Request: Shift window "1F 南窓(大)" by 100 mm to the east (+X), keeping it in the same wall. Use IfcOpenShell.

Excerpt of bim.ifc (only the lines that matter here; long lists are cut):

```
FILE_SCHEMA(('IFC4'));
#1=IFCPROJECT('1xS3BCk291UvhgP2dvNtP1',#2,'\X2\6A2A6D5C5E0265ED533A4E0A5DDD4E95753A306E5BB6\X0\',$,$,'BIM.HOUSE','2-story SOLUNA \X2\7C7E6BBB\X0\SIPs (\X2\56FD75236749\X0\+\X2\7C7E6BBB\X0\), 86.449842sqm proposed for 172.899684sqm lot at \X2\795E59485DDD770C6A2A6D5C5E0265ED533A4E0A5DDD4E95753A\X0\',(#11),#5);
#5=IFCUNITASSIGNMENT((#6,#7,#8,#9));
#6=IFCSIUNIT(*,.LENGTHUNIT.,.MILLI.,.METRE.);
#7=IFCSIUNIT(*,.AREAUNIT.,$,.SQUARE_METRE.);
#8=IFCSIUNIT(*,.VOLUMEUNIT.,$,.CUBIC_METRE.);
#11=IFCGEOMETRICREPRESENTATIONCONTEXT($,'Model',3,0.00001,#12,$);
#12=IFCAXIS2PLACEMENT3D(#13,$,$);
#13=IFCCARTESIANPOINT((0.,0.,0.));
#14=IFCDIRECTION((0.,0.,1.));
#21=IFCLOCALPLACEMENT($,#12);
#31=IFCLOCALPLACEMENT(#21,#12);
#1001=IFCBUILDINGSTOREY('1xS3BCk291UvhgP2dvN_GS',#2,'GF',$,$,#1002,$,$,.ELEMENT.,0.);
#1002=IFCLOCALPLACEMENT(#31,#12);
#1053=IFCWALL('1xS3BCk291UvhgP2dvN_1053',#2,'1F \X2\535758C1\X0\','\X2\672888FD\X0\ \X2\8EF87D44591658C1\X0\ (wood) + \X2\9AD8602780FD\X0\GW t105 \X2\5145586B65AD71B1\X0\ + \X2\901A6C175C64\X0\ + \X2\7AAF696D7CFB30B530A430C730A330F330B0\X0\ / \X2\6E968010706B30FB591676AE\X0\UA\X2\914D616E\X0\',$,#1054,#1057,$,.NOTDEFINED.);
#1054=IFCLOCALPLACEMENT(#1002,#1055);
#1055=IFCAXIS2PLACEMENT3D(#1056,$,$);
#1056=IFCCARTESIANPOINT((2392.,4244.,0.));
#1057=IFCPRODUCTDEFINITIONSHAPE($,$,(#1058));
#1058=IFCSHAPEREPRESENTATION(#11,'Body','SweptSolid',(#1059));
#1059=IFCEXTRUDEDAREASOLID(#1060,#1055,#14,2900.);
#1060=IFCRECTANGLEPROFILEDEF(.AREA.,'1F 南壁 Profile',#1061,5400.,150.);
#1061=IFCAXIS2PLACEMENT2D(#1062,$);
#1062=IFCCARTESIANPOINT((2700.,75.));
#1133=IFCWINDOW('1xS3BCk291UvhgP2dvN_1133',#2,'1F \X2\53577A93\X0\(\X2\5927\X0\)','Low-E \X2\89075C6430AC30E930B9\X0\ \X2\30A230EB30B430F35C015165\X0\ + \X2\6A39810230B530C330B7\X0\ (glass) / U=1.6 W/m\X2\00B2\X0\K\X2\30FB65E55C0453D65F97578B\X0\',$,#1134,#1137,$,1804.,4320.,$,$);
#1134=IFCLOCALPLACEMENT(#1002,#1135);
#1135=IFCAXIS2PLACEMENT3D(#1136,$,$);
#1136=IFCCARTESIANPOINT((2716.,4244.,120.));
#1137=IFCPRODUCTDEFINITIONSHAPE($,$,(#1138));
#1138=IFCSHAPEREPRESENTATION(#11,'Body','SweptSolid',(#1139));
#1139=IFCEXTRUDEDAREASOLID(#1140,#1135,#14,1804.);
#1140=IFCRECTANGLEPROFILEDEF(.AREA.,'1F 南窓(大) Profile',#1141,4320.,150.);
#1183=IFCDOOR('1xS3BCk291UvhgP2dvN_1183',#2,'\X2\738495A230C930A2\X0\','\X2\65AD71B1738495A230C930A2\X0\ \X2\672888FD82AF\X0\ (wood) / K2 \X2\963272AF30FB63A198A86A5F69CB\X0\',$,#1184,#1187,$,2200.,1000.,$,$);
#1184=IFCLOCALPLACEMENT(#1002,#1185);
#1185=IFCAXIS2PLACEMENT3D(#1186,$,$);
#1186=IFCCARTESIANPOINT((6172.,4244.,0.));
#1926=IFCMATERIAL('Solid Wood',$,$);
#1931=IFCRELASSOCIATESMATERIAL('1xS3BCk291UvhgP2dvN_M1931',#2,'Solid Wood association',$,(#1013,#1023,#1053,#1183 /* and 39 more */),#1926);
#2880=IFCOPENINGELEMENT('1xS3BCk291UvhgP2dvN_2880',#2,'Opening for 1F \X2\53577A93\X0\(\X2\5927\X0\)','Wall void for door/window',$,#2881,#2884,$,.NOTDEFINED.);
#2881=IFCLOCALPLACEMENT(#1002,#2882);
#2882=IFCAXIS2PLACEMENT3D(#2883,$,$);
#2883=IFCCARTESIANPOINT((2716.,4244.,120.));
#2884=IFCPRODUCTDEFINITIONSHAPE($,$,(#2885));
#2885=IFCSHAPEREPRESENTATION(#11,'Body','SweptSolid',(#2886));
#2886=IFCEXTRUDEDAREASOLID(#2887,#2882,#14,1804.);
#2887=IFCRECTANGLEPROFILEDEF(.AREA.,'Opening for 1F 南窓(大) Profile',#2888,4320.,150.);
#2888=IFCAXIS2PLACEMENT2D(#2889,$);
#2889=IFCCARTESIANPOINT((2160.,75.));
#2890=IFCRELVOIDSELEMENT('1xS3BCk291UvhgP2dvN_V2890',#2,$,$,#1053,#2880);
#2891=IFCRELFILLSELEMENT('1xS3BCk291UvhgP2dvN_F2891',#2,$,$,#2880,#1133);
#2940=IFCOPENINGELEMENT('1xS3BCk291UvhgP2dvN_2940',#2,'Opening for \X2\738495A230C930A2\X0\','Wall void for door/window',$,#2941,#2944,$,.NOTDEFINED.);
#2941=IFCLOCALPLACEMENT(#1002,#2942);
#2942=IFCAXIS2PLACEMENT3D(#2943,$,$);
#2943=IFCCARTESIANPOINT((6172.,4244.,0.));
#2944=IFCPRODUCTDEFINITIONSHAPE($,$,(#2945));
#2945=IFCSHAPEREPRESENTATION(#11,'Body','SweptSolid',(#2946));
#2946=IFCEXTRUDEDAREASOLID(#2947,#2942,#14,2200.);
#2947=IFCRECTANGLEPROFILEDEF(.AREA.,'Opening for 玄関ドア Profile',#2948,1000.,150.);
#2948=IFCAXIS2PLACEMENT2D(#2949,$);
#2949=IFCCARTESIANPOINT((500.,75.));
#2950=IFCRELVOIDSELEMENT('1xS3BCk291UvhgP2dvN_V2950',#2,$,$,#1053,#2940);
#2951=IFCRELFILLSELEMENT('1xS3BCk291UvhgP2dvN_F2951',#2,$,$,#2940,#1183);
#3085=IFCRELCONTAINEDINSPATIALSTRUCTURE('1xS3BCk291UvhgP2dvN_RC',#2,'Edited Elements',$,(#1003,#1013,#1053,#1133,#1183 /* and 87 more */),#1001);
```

```python
import ifcopenshell
import ifcopenshell.api.geometry
import ifcopenshell.util.placement
import ifcopenshell.util.unit

model = ifcopenshell.open("bim.ifc")
unit_scale = ifcopenshell.util.unit.calculate_unit_scale(model)

window = model.by_guid("1xS3BCk291UvhgP2dvN_1133")
opening = window.FillsVoids[0].RelatingOpeningElement
wall = opening.VoidsElements[0].RelatingBuildingElement

wall_matrix = ifcopenshell.util.placement.get_local_placement(wall.ObjectPlacement)
shift = wall_matrix[:3, 0] * 0.1 / unit_scale
before = ifcopenshell.util.placement.get_local_placement(window.ObjectPlacement)[:3, 3].copy()

# The window is not placed relative to its opening, so move both.
for product in (opening, window):
    matrix = ifcopenshell.util.placement.get_local_placement(product.ObjectPlacement)
    matrix[:3, 3] += shift
    ifcopenshell.api.geometry.edit_object_placement(model, product=product, matrix=matrix, is_si=False)

after = ifcopenshell.util.placement.get_local_placement(window.ObjectPlacement)[:3, 3]
print("window moved by", (after - before).round(3) + 0.0)

model.write("bim-out.ifc")
```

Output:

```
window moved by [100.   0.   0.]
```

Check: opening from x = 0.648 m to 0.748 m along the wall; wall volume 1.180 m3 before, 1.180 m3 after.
